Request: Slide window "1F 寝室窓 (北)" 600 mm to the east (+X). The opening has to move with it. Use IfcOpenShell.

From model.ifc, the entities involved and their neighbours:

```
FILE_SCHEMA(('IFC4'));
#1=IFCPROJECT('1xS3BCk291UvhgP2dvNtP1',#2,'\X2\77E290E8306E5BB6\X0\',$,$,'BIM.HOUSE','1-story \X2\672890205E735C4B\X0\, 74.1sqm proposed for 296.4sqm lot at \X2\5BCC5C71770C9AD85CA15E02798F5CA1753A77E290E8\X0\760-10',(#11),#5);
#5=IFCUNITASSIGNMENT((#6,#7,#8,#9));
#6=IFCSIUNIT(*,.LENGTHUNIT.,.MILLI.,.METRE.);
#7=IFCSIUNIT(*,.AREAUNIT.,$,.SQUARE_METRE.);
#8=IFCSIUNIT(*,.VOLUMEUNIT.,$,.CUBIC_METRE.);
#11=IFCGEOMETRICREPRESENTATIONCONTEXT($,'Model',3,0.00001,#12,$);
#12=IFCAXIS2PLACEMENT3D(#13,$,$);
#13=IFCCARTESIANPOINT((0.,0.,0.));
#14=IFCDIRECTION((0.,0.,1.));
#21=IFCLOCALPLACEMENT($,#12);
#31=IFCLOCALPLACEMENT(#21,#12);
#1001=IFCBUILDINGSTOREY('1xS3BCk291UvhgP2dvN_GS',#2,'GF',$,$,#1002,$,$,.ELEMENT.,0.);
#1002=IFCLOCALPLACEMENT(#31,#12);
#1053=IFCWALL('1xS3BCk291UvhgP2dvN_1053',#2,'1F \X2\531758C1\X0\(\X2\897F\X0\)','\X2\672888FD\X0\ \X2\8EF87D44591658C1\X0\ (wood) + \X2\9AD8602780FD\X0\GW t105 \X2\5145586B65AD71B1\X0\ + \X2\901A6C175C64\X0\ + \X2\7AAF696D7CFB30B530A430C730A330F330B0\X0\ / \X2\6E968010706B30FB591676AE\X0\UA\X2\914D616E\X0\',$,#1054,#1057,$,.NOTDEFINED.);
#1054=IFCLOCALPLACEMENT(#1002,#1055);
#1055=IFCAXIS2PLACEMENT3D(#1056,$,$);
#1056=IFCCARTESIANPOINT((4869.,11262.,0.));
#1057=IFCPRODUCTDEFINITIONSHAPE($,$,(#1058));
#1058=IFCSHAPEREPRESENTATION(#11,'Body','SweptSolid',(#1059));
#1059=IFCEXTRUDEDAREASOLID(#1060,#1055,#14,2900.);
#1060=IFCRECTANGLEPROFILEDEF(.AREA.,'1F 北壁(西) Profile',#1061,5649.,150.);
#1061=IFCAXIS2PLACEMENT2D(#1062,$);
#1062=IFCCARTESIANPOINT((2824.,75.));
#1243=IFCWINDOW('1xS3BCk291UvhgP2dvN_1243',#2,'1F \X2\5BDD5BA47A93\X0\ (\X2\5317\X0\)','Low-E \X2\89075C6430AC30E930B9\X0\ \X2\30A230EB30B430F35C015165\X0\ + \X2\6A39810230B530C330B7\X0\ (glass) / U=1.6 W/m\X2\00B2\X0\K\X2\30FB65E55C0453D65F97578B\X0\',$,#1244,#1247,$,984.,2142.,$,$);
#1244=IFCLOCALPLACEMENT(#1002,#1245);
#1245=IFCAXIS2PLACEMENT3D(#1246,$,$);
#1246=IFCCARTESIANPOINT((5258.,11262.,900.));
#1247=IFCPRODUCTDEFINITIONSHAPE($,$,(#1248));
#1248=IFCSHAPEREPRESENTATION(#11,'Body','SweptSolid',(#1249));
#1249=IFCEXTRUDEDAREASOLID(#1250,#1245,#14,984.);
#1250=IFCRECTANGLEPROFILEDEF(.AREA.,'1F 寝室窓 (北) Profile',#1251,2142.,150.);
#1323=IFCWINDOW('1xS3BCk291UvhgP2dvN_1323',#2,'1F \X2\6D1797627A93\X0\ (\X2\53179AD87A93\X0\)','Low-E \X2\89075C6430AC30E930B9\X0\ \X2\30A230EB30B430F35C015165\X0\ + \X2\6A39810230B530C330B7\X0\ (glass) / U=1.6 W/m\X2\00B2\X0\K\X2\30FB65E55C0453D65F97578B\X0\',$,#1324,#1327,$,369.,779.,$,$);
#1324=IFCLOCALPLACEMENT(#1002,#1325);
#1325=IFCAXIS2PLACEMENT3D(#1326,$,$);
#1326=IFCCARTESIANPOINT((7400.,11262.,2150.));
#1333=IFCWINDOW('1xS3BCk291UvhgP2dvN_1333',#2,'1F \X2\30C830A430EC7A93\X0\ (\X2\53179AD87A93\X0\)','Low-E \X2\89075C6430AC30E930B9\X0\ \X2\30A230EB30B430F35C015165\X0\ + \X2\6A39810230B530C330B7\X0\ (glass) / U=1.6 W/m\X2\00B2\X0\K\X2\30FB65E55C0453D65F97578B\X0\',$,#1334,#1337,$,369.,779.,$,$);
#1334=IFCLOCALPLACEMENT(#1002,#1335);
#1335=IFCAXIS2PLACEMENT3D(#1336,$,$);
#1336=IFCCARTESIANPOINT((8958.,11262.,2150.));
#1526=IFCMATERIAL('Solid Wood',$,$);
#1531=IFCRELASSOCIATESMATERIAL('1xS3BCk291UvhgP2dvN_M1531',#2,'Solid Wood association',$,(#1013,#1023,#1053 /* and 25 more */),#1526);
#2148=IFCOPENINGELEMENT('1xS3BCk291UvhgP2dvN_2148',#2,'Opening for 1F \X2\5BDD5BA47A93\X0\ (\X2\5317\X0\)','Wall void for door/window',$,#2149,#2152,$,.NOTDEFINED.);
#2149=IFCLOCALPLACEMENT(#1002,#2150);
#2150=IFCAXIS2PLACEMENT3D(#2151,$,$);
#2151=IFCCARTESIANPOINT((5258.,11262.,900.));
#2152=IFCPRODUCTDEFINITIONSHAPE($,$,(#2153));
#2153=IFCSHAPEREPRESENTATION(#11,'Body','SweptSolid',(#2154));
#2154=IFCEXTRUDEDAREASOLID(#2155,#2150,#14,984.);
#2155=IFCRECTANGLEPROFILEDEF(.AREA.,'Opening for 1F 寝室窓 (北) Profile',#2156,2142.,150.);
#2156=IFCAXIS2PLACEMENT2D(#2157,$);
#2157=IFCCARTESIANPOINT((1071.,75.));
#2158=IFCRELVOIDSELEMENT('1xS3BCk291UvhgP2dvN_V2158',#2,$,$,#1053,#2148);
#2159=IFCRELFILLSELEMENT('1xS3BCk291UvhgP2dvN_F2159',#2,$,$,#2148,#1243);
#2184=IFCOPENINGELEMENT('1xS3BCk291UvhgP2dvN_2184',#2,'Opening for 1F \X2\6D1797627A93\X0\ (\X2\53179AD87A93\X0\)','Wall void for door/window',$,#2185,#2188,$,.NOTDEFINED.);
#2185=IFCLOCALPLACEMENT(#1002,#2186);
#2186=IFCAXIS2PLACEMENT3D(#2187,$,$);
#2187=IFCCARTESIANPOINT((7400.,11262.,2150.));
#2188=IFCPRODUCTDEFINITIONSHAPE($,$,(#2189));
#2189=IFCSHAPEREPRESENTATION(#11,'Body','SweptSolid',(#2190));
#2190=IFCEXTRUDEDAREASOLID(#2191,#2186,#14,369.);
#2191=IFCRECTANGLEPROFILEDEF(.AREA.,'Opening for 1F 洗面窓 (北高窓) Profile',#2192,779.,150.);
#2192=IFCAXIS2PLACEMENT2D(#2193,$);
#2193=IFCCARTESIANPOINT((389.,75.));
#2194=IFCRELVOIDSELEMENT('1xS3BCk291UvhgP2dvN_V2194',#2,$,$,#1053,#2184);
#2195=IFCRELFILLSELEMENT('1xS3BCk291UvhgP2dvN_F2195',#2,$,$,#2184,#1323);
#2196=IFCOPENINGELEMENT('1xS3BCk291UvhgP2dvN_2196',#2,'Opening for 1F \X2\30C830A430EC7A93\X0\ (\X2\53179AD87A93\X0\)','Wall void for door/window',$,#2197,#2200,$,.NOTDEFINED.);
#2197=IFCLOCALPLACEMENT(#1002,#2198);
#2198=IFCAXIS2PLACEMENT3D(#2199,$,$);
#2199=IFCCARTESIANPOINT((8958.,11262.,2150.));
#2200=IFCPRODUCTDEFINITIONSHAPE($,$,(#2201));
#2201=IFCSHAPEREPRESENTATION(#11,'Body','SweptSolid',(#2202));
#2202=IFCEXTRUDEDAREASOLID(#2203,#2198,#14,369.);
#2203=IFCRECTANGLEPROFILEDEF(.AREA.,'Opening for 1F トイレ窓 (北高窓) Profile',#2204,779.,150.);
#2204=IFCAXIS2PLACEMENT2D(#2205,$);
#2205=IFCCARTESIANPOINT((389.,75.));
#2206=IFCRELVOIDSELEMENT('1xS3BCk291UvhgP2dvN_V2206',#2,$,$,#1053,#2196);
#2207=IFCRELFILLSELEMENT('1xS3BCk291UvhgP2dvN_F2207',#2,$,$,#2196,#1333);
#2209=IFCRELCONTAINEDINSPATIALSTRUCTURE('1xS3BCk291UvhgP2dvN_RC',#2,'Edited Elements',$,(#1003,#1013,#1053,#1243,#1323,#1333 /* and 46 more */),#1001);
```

```python
import ifcopenshell
import ifcopenshell.api.geometry
import ifcopenshell.util.placement
import ifcopenshell.util.unit

model = ifcopenshell.open("model.ifc")
unit_scale = ifcopenshell.util.unit.calculate_unit_scale(model)

window = model.by_guid("1xS3BCk291UvhgP2dvN_1243")
opening = window.FillsVoids[0].RelatingOpeningElement
wall = opening.VoidsElements[0].RelatingBuildingElement

wall_matrix = ifcopenshell.util.placement.get_local_placement(wall.ObjectPlacement)
shift = wall_matrix[:3, 0] * 0.6 / unit_scale
before = ifcopenshell.util.placement.get_local_placement(window.ObjectPlacement)[:3, 3].copy()

# The window is not placed relative to its opening, so move both.
for product in (opening, window):
    matrix = ifcopenshell.util.placement.get_local_placement(product.ObjectPlacement)
    matrix[:3, 3] += shift
    ifcopenshell.api.geometry.edit_object_placement(model, product=product, matrix=matrix, is_si=False)

after = ifcopenshell.util.placement.get_local_placement(window.ObjectPlacement)[:3, 3]
print("window moved by", (after - before).round(3) + 0.0)

model.write("model_rev.ifc")
```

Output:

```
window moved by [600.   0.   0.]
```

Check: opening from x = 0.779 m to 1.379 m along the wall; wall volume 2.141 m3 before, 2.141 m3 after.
